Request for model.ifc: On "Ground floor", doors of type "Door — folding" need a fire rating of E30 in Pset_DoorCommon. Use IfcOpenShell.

First a look at what the model holds.

```python
import ifcopenshell
import ifcopenshell.util.element

model = ifcopenshell.open("model.ifc")
print(model.schema)
storey = next(s for s in model.by_type("IfcBuildingStorey") if s.Name == "Ground floor")
doors = [e for e in ifcopenshell.util.element.get_decomposition(storey) if e.is_a("IfcDoor")]
seen = {}
for e in doors:
    element_type = ifcopenshell.util.element.get_type(e)
    key = (element_type.Name if element_type != e and element_type else None, ifcopenshell.util.element.get_pset(e, "Pset_DoorCommon", "FireRating"))
    seen[key] = seen.get(key, 0) + 1
for (name, value), count in sorted(seen.items(), key=str):
    print(count, "x", name, "|", value)
```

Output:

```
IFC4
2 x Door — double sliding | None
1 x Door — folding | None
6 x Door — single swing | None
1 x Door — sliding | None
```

```python
import ifcopenshell
import ifcopenshell.api.pset
import ifcopenshell.util.element

model = ifcopenshell.open("model.ifc")

storey = next(s for s in model.by_type("IfcBuildingStorey") if s.Name == "Ground floor")
doors = [e for e in ifcopenshell.util.element.get_decomposition(storey) if e.is_a("IfcDoor")]

count = 0
for e in doors:
    element_type = ifcopenshell.util.element.get_type(e)
    if element_type in (None, e) or element_type.Name != "Door — folding":
        continue
    # add_pset returns the element's existing set when there is one.
    pset = ifcopenshell.api.pset.add_pset(model, product=e, name="Pset_DoorCommon")
    ifcopenshell.api.pset.edit_pset(model, pset=pset, properties={"FireRating": "E30"})
    count += 1

print(count, "doors updated")

model.write("model-out.ifc")
```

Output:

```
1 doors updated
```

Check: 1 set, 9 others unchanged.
